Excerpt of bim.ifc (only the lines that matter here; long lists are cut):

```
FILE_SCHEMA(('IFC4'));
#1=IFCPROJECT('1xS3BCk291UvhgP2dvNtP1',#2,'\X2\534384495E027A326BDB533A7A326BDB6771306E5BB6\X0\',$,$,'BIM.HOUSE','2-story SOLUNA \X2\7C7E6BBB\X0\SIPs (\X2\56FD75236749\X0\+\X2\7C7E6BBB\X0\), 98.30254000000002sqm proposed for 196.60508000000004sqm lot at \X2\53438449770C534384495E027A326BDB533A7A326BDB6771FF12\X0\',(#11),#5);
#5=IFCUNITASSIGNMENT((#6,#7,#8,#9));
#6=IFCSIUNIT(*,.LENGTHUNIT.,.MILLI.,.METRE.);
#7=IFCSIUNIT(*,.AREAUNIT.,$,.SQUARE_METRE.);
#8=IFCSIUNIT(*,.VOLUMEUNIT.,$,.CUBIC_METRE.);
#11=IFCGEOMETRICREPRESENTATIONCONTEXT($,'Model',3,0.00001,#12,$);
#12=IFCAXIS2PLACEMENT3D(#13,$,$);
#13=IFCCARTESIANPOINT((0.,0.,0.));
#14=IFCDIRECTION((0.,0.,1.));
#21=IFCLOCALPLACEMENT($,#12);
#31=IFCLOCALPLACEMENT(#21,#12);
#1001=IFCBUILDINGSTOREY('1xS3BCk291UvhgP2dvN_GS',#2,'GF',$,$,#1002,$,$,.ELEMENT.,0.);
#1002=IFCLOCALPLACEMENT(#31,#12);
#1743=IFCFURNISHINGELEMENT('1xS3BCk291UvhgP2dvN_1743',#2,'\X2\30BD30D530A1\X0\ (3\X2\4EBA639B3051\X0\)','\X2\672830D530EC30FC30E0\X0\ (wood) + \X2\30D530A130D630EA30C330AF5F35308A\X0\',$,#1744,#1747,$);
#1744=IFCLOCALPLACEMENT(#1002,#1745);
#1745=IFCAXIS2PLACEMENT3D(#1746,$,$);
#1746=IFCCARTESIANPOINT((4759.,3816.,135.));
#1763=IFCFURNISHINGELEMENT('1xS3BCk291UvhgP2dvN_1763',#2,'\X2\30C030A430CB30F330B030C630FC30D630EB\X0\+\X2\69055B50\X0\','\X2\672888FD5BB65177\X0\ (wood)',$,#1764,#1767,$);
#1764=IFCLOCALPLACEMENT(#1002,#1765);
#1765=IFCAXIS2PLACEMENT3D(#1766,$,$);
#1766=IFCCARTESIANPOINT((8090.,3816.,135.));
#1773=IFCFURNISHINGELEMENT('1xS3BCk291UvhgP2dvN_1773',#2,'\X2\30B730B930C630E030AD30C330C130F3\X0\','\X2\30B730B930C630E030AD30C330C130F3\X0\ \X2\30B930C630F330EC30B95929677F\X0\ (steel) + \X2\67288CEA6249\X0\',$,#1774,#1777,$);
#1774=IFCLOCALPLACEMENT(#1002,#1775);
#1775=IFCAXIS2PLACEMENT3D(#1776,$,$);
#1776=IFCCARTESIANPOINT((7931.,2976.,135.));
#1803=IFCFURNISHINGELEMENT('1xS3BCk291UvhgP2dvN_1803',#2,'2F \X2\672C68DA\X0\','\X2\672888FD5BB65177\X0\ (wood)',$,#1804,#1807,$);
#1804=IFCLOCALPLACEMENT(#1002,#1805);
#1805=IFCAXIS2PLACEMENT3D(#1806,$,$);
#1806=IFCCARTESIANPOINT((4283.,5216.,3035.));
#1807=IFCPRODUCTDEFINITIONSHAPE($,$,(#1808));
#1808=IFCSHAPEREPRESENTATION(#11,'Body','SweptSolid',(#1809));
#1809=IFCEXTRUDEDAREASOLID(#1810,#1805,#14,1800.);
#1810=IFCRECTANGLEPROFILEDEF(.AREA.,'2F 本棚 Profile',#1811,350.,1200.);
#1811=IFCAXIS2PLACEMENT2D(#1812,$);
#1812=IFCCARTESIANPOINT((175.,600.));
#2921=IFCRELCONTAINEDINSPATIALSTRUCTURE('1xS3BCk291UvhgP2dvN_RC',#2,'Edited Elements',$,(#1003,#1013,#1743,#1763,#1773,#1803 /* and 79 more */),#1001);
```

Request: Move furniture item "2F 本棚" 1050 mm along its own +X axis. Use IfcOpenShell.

```python
import ifcopenshell
import ifcopenshell.api.geometry
import ifcopenshell.util.placement
import ifcopenshell.util.unit

model = ifcopenshell.open("bim.ifc")
unit_scale = ifcopenshell.util.unit.calculate_unit_scale(model)

item = model.by_guid("1xS3BCk291UvhgP2dvN_1803")
matrix = ifcopenshell.util.placement.get_local_placement(item.ObjectPlacement)
matrix[:3, 3] += matrix[:3, 0] * 1.05 / unit_scale
ifcopenshell.api.geometry.edit_object_placement(model, product=item, matrix=matrix, is_si=False)

print(ifcopenshell.util.placement.get_local_placement(item.ObjectPlacement).round(3) + 0.0)

model.write("bim_rev.ifc")
```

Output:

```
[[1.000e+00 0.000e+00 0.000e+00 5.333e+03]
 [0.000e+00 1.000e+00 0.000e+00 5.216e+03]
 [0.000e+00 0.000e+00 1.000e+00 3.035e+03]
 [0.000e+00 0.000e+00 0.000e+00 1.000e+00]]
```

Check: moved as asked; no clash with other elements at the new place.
